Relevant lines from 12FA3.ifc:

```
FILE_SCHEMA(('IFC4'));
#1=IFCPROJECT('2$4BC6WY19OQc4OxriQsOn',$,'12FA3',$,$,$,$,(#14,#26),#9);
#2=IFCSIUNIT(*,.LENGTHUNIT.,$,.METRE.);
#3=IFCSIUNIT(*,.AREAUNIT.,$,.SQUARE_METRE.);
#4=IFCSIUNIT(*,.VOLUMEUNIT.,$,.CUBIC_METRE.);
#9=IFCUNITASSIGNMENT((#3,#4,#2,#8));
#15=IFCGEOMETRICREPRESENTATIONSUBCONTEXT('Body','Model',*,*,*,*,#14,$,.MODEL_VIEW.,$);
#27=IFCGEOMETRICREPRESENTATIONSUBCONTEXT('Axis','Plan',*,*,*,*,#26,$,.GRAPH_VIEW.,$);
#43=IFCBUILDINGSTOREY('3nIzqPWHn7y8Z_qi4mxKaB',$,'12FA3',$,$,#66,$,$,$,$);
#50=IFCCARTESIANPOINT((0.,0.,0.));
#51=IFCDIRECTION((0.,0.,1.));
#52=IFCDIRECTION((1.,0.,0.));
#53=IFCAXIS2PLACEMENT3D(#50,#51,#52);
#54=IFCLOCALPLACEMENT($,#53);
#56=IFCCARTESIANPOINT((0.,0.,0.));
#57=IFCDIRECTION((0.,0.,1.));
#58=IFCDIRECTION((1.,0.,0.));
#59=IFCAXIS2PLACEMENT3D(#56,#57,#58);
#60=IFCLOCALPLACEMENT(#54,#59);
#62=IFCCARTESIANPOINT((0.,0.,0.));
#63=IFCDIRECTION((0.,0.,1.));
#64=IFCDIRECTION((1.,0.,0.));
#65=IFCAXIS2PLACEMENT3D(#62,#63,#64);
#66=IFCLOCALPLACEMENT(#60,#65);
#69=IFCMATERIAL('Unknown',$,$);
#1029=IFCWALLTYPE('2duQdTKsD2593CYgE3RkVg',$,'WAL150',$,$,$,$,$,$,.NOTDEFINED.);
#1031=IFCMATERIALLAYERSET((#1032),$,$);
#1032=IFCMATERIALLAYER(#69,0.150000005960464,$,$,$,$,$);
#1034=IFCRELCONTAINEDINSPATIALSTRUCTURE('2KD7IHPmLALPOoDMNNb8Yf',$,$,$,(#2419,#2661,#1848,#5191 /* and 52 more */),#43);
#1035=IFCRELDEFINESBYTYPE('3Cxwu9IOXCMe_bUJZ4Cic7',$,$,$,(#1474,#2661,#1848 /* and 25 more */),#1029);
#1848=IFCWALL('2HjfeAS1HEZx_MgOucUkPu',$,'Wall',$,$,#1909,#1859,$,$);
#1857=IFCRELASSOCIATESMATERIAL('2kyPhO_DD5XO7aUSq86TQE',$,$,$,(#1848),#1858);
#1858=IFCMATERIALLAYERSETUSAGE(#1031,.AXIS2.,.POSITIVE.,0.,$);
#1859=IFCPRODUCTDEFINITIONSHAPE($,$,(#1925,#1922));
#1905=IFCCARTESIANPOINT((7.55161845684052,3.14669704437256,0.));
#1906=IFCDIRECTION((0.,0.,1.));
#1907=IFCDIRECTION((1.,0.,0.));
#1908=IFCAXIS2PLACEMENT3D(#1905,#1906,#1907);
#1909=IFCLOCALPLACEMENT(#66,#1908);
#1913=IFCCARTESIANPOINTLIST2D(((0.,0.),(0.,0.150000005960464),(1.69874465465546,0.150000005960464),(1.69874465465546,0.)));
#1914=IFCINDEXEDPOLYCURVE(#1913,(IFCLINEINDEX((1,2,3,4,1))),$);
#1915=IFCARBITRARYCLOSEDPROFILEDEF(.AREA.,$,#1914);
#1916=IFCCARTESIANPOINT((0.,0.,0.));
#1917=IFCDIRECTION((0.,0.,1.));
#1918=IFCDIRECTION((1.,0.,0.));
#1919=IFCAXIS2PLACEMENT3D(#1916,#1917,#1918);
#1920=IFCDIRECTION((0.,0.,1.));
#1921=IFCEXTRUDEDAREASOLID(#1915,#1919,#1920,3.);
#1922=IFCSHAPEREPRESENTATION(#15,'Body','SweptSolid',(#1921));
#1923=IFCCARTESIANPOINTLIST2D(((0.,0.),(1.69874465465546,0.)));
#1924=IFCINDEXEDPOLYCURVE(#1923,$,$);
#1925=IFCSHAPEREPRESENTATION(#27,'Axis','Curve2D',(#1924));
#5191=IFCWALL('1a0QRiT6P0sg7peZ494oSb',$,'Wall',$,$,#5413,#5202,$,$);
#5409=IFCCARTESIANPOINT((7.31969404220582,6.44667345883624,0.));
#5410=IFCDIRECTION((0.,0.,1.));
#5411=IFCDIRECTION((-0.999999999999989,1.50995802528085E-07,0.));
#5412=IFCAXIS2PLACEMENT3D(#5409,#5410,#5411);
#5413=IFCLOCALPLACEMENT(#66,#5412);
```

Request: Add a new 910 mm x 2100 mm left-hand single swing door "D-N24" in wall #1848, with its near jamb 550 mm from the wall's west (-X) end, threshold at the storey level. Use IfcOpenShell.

```python
import numpy as np
import ifcopenshell
import ifcopenshell.api.feature
import ifcopenshell.api.geometry
import ifcopenshell.api.root
import ifcopenshell.api.spatial
import ifcopenshell.geom
import ifcopenshell.util.element
import ifcopenshell.util.placement
import ifcopenshell.util.representation
import ifcopenshell.util.shape
import ifcopenshell.util.unit

model = ifcopenshell.open("12FA3.ifc")
unit_scale = ifcopenshell.util.unit.calculate_unit_scale(model)
settings = ifcopenshell.geom.settings()


def volume(element):
    """Net volume in cubic metres, openings subtracted."""
    shape = ifcopenshell.geom.create_shape(settings, element)
    return ifcopenshell.util.shape.get_volume(shape.geometry)


wall = model.by_guid("2HjfeAS1HEZx_MgOucUkPu")
storey = ifcopenshell.util.element.get_container(wall, ifc_class="IfcBuildingStorey")
context = ifcopenshell.util.representation.get_context(model, "Model", "Body", "MODEL_VIEW")
before = volume(wall)

width, height, from_end, sill = 0.91, 2.1, 0.55, 0.0  # metres

# The wall runs along its own X axis, and the end named is its -X end.
wall_shape = ifcopenshell.geom.create_shape(settings, wall)
x, y, z = ifcopenshell.util.shape.get_vertices(wall_shape.geometry).T
start = x.min() + from_end
face, thickness = float(y.min()), float(y.max() - y.min())
wall_matrix = ifcopenshell.util.placement.get_local_placement(wall.ObjectPlacement)
level = ifcopenshell.util.placement.get_local_placement(storey.ObjectPlacement)[2, 3]


def in_wall(x, y):
    """Placement at x, y metres in the wall's axes, at sill height."""
    matrix = wall_matrix.copy()
    matrix[:, 3] = wall_matrix @ np.array([x / unit_scale, y / unit_scale, 0.0, 1.0])
    matrix[2, 3] = level + sill / unit_scale
    return matrix


# Opening: a box that overshoots both wall faces by 50 mm.
opening = ifcopenshell.api.root.create_entity(model, ifc_class="IfcOpeningElement", predefined_type="OPENING")
box = ifcopenshell.api.geometry.add_wall_representation(
    model, context=context, length=width, height=height, thickness=thickness + 0.1
)
ifcopenshell.api.geometry.assign_representation(model, product=opening, representation=box)
ifcopenshell.api.geometry.edit_object_placement(model, product=opening, matrix=in_wall(start, face - 0.05), is_si=False)
ifcopenshell.api.feature.add_feature(model, feature=opening, element=wall)

door = ifcopenshell.api.root.create_entity(model, ifc_class="IfcDoor", name="D-N24", predefined_type="DOOR")
door.OverallWidth, door.OverallHeight = width / unit_scale, height / unit_scale
door.OperationType = "SINGLE_SWING_LEFT"
body = ifcopenshell.api.geometry.add_door_representation(
    model,
    context=context,
    overall_width=door.OverallWidth,
    overall_height=door.OverallHeight,
    operation_type="SINGLE_SWING_LEFT",
    lining_properties={"LiningDepth": thickness / unit_scale, "ThresholdDepth": thickness / unit_scale},
)
ifcopenshell.api.geometry.assign_representation(model, product=door, representation=body)
ifcopenshell.api.spatial.assign_container(model, products=[door], relating_structure=storey)
ifcopenshell.api.feature.add_filling(model, opening=opening, element=door)

# The lining spans the wall, so the door starts at the wall face.
ifcopenshell.api.geometry.edit_object_placement(model, product=door, matrix=in_wall(start, face), is_si=False)

after = volume(wall)

print(f"wall volume {before:.3f} -> {after:.3f} m3")

model.write("12FA3_rev.ifc")
```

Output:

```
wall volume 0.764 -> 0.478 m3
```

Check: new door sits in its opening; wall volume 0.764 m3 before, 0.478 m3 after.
